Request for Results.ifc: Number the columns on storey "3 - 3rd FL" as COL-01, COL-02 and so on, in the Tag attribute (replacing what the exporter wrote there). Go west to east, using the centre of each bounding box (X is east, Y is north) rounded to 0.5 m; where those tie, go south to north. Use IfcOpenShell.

First a look at what the model holds.

```python
import ifcopenshell
import ifcopenshell.util.element
import ifcopenshell.util.placement

model = ifcopenshell.open("Results.ifc")
print(model.schema)
storey = next(s for s in model.by_type("IfcBuildingStorey") if s.Name == "3 - 3rd FL")
columns = [e for e in ifcopenshell.util.element.get_decomposition(storey) if e.is_a("IfcColumn")]
for e in sorted(columns, key=lambda e: e.id()):
    origin = ifcopenshell.util.placement.get_local_placement(e.ObjectPlacement)[:3, 3]
    print(e.id(), e.Tag, e.Name, origin.round(2) + 0.0, sep=" | ")
```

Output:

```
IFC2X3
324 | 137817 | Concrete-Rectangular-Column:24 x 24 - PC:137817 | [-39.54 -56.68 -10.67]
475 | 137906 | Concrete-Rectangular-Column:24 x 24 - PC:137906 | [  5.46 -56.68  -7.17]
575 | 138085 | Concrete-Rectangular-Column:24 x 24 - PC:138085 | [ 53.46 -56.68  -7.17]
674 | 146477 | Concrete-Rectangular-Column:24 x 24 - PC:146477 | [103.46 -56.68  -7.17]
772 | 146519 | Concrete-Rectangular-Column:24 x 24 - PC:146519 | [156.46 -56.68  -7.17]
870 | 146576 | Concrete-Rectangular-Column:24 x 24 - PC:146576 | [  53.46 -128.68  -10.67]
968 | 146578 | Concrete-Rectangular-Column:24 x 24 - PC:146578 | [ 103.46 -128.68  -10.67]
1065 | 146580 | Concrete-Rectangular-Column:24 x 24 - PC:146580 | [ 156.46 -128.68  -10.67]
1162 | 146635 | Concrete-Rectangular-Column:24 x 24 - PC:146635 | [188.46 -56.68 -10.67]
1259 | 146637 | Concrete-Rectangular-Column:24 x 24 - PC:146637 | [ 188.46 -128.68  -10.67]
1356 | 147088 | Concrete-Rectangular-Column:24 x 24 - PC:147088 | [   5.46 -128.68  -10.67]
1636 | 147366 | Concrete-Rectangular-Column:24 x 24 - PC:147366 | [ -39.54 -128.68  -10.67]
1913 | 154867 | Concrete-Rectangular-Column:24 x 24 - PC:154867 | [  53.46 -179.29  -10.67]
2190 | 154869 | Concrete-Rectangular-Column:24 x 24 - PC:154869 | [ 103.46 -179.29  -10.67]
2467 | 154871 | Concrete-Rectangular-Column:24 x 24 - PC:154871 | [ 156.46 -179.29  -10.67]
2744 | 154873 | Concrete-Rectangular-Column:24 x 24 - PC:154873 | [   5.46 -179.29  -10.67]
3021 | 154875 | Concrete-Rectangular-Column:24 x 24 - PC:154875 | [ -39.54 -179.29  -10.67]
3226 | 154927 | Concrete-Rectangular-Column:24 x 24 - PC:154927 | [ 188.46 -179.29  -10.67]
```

```python
import ifcopenshell
import ifcopenshell.geom
import ifcopenshell.util.element
import ifcopenshell.util.shape

model = ifcopenshell.open("Results.ifc")
settings = ifcopenshell.geom.settings()
settings.set("use-world-coords", True)


def centre(element):
    shape = ifcopenshell.geom.create_shape(settings, element)
    return ifcopenshell.util.shape.get_bbox_centroid(shape.geometry)


storey = next(s for s in model.by_type("IfcBuildingStorey") if s.Name == "3 - 3rd FL")
columns = [e for e in ifcopenshell.util.element.get_decomposition(storey) if e.is_a("IfcColumn")]

# Insertion points can sit at a corner or the storey origin, so sort by the geometry (in metres).
centres = {e: centre(e) for e in columns}
columns.sort(key=lambda e: (round(centres[e][0] / 0.5), centres[e][1]))

for i, e in enumerate(columns, start=1):
    number = f"COL-{i:02d}"
    e.Tag = number
    print(e.id(), number)

model.write("Results_rev.ifc")
```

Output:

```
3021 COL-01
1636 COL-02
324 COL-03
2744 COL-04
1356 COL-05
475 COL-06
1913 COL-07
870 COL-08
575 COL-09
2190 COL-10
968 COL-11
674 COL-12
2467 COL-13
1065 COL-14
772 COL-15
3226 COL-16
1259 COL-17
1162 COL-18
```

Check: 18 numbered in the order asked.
